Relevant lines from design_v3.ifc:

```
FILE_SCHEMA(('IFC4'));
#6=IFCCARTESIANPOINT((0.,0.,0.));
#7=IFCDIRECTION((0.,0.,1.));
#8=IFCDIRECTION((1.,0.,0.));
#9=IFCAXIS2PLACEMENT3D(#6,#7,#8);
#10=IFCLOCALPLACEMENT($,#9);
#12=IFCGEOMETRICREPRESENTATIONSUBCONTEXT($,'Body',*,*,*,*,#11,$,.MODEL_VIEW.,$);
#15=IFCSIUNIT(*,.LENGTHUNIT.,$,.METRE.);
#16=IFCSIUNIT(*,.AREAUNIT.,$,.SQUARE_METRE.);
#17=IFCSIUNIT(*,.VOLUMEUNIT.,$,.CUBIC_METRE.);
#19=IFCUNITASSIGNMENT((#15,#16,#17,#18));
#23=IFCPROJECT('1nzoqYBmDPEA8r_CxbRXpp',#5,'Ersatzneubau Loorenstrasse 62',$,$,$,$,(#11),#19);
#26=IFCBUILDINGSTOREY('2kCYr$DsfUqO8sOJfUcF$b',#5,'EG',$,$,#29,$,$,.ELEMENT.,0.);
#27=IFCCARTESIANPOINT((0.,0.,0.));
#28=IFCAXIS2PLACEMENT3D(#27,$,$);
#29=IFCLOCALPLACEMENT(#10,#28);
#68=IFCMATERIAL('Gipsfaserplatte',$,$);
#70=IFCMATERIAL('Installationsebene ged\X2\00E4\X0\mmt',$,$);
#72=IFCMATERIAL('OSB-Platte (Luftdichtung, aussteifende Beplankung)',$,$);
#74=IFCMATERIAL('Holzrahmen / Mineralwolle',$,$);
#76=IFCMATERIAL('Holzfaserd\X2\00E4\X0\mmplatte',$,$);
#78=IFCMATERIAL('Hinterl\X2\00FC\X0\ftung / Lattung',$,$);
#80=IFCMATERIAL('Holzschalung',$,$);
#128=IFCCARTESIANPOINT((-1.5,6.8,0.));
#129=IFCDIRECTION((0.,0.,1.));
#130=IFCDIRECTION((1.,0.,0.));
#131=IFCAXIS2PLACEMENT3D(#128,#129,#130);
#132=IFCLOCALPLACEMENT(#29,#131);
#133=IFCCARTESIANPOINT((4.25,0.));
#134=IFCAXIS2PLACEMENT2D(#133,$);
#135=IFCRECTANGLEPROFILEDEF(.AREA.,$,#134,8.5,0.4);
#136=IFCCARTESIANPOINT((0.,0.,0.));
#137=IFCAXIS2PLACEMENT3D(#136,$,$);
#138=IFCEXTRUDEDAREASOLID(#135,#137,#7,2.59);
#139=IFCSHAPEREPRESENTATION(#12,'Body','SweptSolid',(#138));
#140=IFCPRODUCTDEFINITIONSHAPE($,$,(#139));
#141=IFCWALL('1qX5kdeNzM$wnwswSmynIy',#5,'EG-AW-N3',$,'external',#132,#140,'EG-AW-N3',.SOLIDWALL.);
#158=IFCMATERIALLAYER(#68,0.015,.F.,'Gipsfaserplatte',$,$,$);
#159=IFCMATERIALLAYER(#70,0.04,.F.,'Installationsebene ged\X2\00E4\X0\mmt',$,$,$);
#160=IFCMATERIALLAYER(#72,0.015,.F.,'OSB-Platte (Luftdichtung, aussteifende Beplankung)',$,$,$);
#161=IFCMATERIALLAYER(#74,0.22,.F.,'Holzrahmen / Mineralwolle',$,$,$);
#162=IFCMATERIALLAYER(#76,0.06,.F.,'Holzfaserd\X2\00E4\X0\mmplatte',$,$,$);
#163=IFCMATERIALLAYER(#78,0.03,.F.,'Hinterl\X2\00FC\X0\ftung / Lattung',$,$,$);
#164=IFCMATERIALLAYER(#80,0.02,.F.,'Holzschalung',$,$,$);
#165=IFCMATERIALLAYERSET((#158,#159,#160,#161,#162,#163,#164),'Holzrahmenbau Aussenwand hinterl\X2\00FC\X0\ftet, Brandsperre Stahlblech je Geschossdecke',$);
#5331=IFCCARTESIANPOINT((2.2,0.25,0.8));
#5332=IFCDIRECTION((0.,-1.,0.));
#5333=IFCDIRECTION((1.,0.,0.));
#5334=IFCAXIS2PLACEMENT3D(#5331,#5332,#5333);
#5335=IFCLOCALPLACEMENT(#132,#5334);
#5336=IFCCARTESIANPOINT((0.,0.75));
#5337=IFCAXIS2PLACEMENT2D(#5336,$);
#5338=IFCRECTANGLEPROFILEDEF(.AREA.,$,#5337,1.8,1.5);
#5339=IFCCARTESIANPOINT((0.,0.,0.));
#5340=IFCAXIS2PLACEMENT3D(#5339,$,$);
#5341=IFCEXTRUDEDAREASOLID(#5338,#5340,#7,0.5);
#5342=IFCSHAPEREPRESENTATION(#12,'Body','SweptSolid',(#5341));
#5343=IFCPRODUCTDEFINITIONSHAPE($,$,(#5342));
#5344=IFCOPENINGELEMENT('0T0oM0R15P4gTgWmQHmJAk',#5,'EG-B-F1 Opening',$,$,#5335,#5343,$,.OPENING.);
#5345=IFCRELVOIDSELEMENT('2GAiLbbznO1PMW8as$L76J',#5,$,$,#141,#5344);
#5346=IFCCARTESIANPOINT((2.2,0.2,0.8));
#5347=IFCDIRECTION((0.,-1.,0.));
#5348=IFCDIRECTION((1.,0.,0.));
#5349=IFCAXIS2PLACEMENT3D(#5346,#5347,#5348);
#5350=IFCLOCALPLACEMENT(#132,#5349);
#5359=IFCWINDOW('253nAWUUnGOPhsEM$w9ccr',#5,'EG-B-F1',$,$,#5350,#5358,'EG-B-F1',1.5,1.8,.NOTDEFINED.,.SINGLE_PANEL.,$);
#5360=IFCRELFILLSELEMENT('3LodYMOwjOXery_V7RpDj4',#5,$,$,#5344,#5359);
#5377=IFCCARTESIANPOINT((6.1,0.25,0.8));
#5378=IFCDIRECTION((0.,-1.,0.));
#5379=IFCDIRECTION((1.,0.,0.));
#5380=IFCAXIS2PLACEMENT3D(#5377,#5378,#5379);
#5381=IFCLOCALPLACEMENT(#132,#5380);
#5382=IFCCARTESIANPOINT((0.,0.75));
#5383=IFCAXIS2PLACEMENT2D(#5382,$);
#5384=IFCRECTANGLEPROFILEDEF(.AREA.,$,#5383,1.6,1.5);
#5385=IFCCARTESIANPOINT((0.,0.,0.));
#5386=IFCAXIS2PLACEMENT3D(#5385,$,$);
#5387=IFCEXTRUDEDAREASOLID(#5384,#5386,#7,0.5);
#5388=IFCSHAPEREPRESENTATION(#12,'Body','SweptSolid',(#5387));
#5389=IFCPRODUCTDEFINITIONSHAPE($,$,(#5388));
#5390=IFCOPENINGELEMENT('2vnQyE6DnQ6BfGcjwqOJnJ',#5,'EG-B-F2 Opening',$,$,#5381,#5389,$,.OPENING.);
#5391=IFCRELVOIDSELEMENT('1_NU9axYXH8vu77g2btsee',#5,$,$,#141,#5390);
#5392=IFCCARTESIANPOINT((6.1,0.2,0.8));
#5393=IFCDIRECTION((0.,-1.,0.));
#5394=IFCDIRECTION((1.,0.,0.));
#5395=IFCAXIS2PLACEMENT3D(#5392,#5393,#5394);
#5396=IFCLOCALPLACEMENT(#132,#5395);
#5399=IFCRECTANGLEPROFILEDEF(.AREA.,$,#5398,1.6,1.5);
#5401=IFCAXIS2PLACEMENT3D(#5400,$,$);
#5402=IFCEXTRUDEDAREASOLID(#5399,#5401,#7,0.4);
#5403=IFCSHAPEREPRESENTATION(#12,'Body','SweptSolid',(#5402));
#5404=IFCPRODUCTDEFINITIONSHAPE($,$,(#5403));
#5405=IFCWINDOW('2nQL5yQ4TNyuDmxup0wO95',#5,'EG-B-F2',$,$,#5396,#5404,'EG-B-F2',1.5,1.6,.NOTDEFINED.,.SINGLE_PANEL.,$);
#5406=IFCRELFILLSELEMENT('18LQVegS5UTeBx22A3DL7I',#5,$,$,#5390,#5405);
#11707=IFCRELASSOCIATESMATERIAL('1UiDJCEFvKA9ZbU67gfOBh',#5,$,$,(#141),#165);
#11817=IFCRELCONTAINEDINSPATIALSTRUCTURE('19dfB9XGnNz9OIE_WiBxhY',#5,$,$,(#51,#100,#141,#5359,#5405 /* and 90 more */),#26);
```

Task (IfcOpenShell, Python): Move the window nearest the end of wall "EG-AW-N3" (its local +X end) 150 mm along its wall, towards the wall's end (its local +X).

```python
import ifcopenshell
import ifcopenshell.api.geometry
import ifcopenshell.util.placement
import ifcopenshell.util.unit

model = ifcopenshell.open("design_v3.ifc")
unit_scale = ifcopenshell.util.unit.calculate_unit_scale(model)

window = model.by_guid("2nQL5yQ4TNyuDmxup0wO95")
opening = window.FillsVoids[0].RelatingOpeningElement
wall = opening.VoidsElements[0].RelatingBuildingElement

wall_matrix = ifcopenshell.util.placement.get_local_placement(wall.ObjectPlacement)
shift = wall_matrix[:3, 0] * 0.15 / unit_scale
before = ifcopenshell.util.placement.get_local_placement(window.ObjectPlacement)[:3, 3].copy()

# The window is not placed relative to its opening, so move both.
for product in (opening, window):
    matrix = ifcopenshell.util.placement.get_local_placement(product.ObjectPlacement)
    matrix[:3, 3] += shift
    ifcopenshell.api.geometry.edit_object_placement(model, product=product, matrix=matrix, is_si=False)

after = ifcopenshell.util.placement.get_local_placement(window.ObjectPlacement)[:3, 3]
print("window moved by", (after - before).round(3) + 0.0)

model.write("design_v3-out.ifc")
```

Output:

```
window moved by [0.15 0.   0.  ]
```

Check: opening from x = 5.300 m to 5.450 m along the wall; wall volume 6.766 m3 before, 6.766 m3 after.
